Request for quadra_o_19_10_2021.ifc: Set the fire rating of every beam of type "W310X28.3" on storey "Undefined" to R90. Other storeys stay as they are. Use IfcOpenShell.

First a look at what the model holds.

```python
import ifcopenshell
import ifcopenshell.util.element

model = ifcopenshell.open("quadra_o_19_10_2021.ifc")
print(model.schema)
storey = next(s for s in model.by_type("IfcBuildingStorey") if s.Name == "Undefined")
beams = [e for e in ifcopenshell.util.element.get_decomposition(storey) if e.is_a("IfcBeam")]
seen = {}
for e in beams:
    element_type = ifcopenshell.util.element.get_type(e)
    key = (element_type.Name if element_type != e and element_type else None, ifcopenshell.util.element.get_pset(e, "Pset_BeamCommon", "FireRating"))
    seen[key] = seen.get(key, 0) + 1
for (name, value), count in sorted(seen.items(), key=str):
    print(count, "x", name, "|", value)
```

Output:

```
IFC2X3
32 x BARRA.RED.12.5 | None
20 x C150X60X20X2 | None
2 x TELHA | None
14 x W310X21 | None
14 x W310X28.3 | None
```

```python
import ifcopenshell
import ifcopenshell.api.pset
import ifcopenshell.util.element

model = ifcopenshell.open("quadra_o_19_10_2021.ifc")

storey = next(s for s in model.by_type("IfcBuildingStorey") if s.Name == "Undefined")
beams = [e for e in ifcopenshell.util.element.get_decomposition(storey) if e.is_a("IfcBeam")]

count = 0
for e in beams:
    element_type = ifcopenshell.util.element.get_type(e)
    if element_type in (None, e) or element_type.Name != "W310X28.3":
        continue
    found = ifcopenshell.util.element.get_pset(e, "Pset_BeamCommon", should_inherit=False)
    if found:
        pset = model.by_id(found["id"])
        if len(ifcopenshell.util.element.get_elements_by_pset(pset)) > 1:
            pset = ifcopenshell.api.pset.unshare_pset(model, products=[e], pset=pset)[0]
    else:
        pset = ifcopenshell.api.pset.add_pset(model, product=e, name="Pset_BeamCommon")
    ifcopenshell.api.pset.edit_pset(model, pset=pset, properties={"FireRating": "R90"})
    count += 1

print(count, "beams updated")

model.write("quadra_o_19_10_2021_rev.ifc")
```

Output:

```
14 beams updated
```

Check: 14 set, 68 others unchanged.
